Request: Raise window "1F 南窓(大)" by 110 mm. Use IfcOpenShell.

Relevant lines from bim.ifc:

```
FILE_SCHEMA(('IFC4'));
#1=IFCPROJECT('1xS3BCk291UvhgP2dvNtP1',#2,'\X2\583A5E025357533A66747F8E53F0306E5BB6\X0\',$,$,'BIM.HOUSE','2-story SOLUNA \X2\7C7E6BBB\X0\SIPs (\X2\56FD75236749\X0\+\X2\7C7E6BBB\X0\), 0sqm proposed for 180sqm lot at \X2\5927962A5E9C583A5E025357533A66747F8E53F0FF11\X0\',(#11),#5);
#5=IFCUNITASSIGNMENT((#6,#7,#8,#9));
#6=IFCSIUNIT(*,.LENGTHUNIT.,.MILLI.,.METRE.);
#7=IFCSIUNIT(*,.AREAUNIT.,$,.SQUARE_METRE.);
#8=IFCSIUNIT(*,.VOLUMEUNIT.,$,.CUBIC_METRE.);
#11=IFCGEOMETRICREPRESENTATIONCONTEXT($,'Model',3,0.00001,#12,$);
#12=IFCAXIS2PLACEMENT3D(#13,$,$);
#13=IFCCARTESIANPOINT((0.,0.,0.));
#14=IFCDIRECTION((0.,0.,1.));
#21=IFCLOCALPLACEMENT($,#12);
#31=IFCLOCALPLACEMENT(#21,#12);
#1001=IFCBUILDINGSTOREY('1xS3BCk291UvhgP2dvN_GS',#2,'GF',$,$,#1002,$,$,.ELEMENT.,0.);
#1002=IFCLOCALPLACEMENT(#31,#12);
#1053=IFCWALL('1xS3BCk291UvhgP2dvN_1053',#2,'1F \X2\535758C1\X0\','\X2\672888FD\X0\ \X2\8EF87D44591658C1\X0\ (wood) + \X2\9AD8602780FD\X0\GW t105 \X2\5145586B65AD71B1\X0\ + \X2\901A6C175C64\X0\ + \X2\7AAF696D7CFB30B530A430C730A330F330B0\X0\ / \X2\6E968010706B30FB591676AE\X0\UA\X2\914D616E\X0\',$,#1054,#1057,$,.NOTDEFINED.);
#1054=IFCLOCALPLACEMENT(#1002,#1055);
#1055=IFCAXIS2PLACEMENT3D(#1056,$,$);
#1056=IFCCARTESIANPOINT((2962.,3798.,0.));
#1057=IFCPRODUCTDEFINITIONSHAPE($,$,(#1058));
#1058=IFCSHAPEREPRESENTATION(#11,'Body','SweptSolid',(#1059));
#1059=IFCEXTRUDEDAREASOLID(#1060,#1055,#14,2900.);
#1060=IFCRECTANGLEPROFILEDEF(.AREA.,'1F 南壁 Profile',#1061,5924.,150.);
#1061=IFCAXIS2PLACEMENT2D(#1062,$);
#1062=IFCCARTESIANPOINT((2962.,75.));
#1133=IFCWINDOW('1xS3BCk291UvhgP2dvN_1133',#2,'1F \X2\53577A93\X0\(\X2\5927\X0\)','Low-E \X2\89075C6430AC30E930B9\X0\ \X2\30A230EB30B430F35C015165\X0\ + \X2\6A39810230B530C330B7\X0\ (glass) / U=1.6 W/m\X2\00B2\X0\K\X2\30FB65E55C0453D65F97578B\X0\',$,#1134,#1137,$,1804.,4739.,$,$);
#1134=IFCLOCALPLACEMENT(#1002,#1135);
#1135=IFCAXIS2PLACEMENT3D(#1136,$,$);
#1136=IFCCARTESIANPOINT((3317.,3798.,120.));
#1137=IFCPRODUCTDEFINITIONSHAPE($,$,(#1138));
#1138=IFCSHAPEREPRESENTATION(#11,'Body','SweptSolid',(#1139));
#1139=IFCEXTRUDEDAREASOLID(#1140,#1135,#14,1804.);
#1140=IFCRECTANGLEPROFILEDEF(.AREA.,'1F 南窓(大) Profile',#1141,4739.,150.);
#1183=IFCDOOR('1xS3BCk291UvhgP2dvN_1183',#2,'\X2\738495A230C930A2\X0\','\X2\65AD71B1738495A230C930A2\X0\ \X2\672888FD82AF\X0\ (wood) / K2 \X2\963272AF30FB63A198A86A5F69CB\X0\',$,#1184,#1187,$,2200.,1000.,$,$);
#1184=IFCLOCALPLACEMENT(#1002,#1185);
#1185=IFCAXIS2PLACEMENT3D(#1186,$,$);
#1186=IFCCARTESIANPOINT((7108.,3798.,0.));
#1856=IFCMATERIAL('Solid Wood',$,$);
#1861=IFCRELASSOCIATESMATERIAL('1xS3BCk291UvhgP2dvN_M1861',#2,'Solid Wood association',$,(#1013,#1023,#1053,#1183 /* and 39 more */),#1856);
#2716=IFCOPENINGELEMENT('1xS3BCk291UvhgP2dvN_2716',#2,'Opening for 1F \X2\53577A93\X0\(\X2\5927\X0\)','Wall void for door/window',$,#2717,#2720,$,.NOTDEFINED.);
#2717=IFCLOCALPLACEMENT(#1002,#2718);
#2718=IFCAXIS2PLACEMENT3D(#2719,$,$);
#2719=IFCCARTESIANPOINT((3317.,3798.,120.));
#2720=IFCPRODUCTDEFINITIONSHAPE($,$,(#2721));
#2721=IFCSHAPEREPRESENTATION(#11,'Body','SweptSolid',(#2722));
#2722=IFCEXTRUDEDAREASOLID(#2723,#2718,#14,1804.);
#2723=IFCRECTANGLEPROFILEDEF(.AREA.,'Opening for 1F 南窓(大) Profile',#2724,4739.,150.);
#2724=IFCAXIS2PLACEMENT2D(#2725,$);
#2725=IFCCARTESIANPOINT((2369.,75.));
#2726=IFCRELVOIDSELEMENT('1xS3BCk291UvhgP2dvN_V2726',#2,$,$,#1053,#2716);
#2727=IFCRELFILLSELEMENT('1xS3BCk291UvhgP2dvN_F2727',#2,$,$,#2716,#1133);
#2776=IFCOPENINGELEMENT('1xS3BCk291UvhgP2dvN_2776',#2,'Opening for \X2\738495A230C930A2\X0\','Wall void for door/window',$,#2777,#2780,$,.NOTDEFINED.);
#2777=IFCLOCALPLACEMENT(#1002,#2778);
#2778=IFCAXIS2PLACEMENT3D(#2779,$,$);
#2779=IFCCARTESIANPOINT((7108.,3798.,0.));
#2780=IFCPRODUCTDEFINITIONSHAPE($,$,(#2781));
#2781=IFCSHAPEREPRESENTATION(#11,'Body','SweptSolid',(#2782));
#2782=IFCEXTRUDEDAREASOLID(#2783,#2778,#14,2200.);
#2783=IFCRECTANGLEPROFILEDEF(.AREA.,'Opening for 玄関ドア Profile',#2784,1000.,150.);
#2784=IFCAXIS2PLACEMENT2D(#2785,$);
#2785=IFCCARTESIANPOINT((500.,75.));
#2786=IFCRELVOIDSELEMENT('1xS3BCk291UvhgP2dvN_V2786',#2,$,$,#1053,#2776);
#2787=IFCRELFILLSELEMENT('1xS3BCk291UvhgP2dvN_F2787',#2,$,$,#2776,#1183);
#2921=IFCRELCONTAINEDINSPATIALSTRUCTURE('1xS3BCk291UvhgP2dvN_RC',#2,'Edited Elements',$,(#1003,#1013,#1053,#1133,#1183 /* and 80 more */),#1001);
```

```python
import numpy as np
import ifcopenshell
import ifcopenshell.api.geometry
import ifcopenshell.util.placement
import ifcopenshell.util.unit

model = ifcopenshell.open("bim.ifc")
unit_scale = ifcopenshell.util.unit.calculate_unit_scale(model)

window = model.by_id(1133)
opening = window.FillsVoids[0].RelatingOpeningElement
dz = 0.11 / unit_scale

shift = np.array([0.0, 0.0, dz])
# The window is not placed relative to its opening, so move both.
for product in (opening, window):
    matrix = ifcopenshell.util.placement.get_local_placement(product.ObjectPlacement)
    matrix[:3, 3] += shift
    ifcopenshell.api.geometry.edit_object_placement(model, product=product, matrix=matrix, is_si=False)

print(f"moved by {dz * unit_scale:+.3f} m")

model.write("bim_updated.ifc")
```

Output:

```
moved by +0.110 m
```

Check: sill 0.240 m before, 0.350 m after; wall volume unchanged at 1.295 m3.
